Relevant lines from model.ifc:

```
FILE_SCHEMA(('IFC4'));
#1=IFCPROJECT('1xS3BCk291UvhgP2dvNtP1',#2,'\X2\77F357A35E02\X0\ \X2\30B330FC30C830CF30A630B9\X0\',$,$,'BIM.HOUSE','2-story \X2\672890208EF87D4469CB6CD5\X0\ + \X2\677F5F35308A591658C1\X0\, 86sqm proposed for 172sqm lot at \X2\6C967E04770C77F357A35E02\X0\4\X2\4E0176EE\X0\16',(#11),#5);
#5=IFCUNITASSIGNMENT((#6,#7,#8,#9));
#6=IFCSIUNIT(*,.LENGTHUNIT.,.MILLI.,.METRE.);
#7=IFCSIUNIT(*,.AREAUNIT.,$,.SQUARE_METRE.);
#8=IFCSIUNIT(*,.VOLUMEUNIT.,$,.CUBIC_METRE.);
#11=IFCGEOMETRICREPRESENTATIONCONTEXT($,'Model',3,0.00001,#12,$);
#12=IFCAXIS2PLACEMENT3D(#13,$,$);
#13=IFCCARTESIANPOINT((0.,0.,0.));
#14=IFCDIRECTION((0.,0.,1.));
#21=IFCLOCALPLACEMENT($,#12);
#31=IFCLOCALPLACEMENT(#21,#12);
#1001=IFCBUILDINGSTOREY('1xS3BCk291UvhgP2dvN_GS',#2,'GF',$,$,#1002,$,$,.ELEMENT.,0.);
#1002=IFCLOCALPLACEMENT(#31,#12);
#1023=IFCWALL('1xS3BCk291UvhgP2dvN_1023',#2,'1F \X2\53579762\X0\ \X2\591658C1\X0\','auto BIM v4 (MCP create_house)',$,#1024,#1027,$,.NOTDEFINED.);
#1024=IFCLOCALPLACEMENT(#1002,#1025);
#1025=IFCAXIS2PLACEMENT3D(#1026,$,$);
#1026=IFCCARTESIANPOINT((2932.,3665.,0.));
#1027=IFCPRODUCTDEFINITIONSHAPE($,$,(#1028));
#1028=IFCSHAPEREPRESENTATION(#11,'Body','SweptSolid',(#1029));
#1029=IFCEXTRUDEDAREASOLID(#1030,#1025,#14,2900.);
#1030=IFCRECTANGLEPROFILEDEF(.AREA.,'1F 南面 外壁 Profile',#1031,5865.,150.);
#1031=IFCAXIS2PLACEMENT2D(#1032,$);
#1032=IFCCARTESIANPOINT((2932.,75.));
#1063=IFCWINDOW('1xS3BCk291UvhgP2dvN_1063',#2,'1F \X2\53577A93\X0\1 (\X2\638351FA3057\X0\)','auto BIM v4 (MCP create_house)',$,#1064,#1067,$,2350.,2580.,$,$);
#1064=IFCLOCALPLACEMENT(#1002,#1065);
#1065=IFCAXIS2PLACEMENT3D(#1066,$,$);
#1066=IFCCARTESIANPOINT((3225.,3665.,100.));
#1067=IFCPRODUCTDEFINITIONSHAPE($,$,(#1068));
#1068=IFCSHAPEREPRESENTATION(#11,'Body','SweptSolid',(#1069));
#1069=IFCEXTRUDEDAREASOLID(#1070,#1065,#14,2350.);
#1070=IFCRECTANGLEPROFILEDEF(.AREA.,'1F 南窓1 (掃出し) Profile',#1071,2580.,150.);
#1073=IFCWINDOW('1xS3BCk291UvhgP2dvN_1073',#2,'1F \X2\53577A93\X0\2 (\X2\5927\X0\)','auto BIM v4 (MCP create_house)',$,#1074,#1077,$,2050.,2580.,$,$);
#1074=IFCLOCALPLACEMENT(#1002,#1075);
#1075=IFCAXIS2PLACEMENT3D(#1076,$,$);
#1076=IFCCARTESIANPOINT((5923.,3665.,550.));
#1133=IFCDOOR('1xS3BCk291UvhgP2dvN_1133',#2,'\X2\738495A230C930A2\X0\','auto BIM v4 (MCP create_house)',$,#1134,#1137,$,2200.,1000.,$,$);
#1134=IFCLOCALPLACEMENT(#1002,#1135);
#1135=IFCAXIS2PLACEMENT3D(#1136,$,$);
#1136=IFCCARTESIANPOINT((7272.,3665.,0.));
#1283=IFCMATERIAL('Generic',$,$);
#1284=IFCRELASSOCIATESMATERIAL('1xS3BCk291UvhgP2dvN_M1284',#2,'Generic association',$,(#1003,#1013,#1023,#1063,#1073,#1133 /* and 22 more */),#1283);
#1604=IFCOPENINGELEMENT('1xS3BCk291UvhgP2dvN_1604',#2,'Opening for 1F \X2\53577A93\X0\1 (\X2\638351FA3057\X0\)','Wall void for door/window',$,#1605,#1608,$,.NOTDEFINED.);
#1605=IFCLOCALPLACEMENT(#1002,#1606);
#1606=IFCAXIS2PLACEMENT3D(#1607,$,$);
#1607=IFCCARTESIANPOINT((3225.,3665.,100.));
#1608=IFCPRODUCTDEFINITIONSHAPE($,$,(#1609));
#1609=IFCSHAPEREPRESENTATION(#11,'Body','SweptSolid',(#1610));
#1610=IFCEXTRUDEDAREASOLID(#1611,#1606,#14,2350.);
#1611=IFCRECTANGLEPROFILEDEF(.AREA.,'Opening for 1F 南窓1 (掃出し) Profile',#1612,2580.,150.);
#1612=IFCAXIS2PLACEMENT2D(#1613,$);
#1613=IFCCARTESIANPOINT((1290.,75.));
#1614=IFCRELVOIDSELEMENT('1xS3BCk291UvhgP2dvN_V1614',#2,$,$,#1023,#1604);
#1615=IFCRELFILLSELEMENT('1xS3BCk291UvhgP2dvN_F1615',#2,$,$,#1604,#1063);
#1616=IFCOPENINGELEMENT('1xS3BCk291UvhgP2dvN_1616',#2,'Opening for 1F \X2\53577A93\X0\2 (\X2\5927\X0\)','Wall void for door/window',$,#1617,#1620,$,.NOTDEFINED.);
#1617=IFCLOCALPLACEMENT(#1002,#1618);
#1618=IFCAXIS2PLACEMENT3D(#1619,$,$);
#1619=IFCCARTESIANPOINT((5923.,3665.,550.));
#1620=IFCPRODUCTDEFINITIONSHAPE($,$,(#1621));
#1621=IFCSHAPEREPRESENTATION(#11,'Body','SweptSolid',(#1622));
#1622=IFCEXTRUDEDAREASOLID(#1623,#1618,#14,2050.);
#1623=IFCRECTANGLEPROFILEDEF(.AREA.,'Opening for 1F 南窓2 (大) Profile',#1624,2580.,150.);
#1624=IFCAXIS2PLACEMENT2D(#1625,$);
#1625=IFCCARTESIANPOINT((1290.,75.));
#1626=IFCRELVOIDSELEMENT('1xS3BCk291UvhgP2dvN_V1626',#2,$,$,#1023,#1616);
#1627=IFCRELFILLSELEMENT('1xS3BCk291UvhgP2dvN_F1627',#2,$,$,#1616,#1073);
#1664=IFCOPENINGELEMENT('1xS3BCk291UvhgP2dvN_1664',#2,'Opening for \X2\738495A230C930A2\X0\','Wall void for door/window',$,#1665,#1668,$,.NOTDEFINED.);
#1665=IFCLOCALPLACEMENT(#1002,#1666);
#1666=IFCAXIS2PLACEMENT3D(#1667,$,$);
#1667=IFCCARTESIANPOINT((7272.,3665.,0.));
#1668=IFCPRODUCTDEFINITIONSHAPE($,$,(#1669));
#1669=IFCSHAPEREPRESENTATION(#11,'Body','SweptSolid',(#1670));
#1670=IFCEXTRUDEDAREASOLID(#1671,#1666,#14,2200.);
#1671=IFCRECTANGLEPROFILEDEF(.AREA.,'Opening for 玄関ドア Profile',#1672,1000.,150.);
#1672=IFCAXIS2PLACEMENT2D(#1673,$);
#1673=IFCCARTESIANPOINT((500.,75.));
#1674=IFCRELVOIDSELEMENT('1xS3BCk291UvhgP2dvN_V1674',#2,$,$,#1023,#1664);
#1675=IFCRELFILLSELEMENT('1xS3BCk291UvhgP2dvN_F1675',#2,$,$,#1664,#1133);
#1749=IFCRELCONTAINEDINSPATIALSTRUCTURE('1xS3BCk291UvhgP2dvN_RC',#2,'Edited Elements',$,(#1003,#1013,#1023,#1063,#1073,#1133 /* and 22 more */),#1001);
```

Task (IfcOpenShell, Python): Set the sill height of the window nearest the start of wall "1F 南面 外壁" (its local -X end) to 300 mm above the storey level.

```python
import numpy as np
import ifcopenshell
import ifcopenshell.api.geometry
import ifcopenshell.geom
import ifcopenshell.util.element
import ifcopenshell.util.placement
import ifcopenshell.util.shape
import ifcopenshell.util.unit

model = ifcopenshell.open("model.ifc")
unit_scale = ifcopenshell.util.unit.calculate_unit_scale(model)

window = model.by_id(1063)
opening = window.FillsVoids[0].RelatingOpeningElement
storey = ifcopenshell.util.element.get_container(window, ifc_class="IfcBuildingStorey")
level = ifcopenshell.util.placement.get_local_placement(storey.ObjectPlacement)[2, 3]

# The opening's origin need not be at the sill, so measure its lowest point.
shape = ifcopenshell.geom.create_shape(ifcopenshell.geom.settings(), opening)
bottom = ifcopenshell.util.shape.get_shape_bottom_elevation(shape, shape.geometry) / unit_scale
dz = level + 0.3 / unit_scale - bottom

shift = np.array([0.0, 0.0, dz])
# The window is not placed relative to its opening, so move both.
for product in (opening, window):
    matrix = ifcopenshell.util.placement.get_local_placement(product.ObjectPlacement)
    matrix[:3, 3] += shift
    ifcopenshell.api.geometry.edit_object_placement(model, product=product, matrix=matrix, is_si=False)

print(f"moved by {dz * unit_scale:+.3f} m")

model.write("model_v2.ifc")
```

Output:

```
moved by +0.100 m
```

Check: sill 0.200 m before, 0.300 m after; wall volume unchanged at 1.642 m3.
